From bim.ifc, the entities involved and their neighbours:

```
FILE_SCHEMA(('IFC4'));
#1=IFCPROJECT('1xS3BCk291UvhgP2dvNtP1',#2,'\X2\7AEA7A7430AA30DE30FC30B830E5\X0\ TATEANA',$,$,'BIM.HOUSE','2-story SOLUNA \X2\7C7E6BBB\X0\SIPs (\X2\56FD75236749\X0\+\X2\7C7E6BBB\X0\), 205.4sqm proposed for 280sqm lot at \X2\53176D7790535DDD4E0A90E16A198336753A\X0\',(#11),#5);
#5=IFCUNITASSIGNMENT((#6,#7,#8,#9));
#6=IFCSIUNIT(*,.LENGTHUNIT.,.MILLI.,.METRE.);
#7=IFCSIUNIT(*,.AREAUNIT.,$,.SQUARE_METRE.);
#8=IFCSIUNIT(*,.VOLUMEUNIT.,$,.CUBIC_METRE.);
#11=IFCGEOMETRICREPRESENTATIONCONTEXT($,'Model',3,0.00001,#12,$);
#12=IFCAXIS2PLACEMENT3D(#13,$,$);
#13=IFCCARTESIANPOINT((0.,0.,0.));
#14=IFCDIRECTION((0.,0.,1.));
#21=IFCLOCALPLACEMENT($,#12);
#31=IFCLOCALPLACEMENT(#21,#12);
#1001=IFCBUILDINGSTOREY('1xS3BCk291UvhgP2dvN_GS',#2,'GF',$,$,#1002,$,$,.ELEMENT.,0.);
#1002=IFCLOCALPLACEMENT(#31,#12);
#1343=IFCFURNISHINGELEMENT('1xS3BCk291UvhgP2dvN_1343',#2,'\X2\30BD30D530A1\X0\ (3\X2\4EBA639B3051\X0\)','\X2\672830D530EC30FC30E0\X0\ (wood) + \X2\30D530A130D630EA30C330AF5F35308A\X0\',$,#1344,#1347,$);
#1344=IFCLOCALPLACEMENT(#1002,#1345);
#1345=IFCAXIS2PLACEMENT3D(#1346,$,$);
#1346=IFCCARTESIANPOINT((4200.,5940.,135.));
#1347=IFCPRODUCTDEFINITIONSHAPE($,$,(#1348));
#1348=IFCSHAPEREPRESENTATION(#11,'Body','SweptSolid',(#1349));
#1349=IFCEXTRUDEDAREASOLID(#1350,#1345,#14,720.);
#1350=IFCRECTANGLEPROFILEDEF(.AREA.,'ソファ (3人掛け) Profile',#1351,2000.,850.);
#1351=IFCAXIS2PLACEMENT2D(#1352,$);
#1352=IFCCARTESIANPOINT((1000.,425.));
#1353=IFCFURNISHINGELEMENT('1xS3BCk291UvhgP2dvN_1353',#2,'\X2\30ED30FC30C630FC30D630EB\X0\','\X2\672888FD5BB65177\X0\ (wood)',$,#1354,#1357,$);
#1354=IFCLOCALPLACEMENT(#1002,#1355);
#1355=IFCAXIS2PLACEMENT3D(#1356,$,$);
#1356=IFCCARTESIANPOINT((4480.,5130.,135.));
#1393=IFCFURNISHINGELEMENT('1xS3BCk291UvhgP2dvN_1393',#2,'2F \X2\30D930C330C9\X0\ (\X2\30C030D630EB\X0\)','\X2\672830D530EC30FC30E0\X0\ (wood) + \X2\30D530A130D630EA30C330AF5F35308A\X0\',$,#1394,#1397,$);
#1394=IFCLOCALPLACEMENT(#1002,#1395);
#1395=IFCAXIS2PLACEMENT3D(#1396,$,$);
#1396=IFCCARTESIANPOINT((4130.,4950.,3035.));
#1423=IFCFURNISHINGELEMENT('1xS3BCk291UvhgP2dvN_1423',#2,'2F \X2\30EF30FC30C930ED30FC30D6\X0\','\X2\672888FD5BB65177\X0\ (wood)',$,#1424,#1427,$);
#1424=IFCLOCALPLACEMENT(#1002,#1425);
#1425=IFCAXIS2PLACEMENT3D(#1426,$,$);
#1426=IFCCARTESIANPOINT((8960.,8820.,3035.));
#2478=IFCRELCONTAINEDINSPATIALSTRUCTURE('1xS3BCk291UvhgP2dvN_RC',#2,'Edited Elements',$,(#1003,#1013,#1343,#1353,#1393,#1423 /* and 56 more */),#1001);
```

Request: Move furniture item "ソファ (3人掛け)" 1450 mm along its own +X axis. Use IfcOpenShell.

```python
import ifcopenshell
import ifcopenshell.api.geometry
import ifcopenshell.util.placement
import ifcopenshell.util.unit

model = ifcopenshell.open("bim.ifc")
unit_scale = ifcopenshell.util.unit.calculate_unit_scale(model)

item = model.by_guid("1xS3BCk291UvhgP2dvN_1343")
matrix = ifcopenshell.util.placement.get_local_placement(item.ObjectPlacement)
matrix[:3, 3] += matrix[:3, 0] * 1.45 / unit_scale
ifcopenshell.api.geometry.edit_object_placement(model, product=item, matrix=matrix, is_si=False)

print(ifcopenshell.util.placement.get_local_placement(item.ObjectPlacement).round(3) + 0.0)

model.write("bim-out.ifc")
```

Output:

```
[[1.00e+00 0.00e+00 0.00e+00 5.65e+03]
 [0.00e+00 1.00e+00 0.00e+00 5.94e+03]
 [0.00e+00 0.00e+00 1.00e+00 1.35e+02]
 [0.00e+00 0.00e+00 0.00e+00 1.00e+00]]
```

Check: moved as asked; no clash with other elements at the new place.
